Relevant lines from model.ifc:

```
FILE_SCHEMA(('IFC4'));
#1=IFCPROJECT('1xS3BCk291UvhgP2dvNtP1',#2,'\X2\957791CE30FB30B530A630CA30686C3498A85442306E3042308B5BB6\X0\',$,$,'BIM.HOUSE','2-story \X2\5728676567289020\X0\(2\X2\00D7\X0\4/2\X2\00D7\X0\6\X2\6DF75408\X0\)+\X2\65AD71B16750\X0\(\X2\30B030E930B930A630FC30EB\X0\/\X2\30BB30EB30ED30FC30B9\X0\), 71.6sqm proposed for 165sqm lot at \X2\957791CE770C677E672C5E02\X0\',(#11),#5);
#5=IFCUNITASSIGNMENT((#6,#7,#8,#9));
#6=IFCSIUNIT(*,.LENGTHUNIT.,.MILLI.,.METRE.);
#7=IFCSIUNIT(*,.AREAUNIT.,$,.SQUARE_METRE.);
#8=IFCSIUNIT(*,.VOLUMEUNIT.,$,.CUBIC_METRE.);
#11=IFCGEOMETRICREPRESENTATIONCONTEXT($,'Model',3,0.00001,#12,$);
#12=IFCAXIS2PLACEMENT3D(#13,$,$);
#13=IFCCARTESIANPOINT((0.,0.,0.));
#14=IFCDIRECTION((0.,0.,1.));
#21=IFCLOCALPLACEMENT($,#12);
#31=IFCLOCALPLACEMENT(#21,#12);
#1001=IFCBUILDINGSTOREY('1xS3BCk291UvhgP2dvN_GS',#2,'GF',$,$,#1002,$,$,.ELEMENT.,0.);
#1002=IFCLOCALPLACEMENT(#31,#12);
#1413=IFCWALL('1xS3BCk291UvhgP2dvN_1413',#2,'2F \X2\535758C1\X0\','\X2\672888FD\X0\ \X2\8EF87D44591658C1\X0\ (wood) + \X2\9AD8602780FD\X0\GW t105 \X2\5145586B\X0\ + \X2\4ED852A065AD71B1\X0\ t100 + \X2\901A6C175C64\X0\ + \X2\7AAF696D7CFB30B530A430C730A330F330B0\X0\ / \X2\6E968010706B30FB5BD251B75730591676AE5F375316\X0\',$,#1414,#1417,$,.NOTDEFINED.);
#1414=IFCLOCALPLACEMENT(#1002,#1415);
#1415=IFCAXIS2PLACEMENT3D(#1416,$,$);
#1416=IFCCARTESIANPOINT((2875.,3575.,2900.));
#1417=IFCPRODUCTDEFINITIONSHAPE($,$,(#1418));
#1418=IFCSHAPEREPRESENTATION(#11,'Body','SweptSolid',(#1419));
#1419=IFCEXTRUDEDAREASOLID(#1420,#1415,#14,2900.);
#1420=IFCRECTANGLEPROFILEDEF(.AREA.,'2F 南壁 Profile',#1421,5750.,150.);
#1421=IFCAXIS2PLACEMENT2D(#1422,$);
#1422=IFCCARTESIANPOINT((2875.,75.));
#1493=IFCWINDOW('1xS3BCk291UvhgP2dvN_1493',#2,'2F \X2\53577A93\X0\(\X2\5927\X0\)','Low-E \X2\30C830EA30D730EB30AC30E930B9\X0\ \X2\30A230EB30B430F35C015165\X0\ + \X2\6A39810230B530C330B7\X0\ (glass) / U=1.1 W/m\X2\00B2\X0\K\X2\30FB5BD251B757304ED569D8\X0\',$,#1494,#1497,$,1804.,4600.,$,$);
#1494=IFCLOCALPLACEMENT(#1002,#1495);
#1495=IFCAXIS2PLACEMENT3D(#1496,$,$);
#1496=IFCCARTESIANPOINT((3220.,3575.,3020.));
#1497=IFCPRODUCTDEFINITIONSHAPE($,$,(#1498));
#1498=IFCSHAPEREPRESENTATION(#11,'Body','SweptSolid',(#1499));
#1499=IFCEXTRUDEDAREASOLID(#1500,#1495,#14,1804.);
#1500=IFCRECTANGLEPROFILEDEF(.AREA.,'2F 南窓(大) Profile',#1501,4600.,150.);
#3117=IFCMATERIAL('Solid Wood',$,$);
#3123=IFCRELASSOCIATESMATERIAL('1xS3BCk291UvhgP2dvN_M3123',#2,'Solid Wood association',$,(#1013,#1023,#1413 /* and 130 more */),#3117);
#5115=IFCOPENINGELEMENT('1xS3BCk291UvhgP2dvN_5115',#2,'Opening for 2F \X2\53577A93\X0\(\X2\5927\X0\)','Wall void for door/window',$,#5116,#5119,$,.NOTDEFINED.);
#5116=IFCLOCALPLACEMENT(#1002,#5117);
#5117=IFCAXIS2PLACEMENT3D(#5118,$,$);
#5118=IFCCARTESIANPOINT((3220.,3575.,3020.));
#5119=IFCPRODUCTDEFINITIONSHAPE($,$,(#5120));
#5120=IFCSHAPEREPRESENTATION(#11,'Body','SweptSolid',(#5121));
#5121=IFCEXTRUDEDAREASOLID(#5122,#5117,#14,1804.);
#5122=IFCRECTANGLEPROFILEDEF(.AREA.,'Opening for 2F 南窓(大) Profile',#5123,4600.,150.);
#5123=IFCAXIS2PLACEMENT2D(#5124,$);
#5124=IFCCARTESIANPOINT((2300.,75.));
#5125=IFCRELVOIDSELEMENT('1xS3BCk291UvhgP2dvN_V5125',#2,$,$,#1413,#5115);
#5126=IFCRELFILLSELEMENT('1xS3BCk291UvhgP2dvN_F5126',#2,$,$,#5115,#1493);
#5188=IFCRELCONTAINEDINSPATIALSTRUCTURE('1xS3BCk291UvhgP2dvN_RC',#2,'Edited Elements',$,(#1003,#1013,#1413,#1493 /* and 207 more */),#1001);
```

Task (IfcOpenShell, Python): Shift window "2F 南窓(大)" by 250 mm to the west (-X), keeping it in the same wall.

```python
import ifcopenshell
import ifcopenshell.api.geometry
import ifcopenshell.util.placement

model = ifcopenshell.open("model.ifc")

window = model.by_guid("1xS3BCk291UvhgP2dvN_1493")
opening = window.FillsVoids[0].RelatingOpeningElement
wall = opening.VoidsElements[0].RelatingBuildingElement

wall_matrix = ifcopenshell.util.placement.get_local_placement(wall.ObjectPlacement)
shift = wall_matrix[:3, 0] * -250.0
before = ifcopenshell.util.placement.get_local_placement(window.ObjectPlacement)[:3, 3].copy()

# The window is not placed relative to its opening, so move both.
for product in (opening, window):
    matrix = ifcopenshell.util.placement.get_local_placement(product.ObjectPlacement)
    matrix[:3, 3] += shift
    ifcopenshell.api.geometry.edit_object_placement(model, product=product, matrix=matrix, is_si=False)

after = ifcopenshell.util.placement.get_local_placement(window.ObjectPlacement)[:3, 3]
print("window moved by", (after - before).round(3) + 0.0)

model.write("model-out.ifc")
```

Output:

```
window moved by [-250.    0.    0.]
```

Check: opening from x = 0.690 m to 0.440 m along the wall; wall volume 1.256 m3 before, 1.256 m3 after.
